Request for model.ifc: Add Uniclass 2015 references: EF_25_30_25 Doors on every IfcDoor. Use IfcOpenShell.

First a look at what the model holds.

```python
import ifcopenshell

model = ifcopenshell.open("model.ifc")
print(model.schema)
print("classifications:", [c.Name for c in model.by_type("IfcClassification")])
for ifc_class in ("IfcDoor", "IfcRoof", "IfcStair", "IfcWall", "IfcWindow"):
    print(ifc_class, len(model.by_type(ifc_class)))
```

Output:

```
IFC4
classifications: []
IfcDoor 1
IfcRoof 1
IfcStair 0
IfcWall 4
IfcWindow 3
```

```python
import ifcopenshell
import ifcopenshell.api.classification

model = ifcopenshell.open("model.ifc")

system = ifcopenshell.api.classification.add_classification(model, classification="Uniclass 2015")

codes = {
    "IfcDoor": ("EF_25_30_25", "Doors"),
}
for ifc_class, (code, name) in codes.items():
    products = model.by_type(ifc_class)
    ifcopenshell.api.classification.add_reference(
        model, products=products, classification=system, identification=code, name=name
    )
    print(code, len(products))

model.write("model-out.ifc")
```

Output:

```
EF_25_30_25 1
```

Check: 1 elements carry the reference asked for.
